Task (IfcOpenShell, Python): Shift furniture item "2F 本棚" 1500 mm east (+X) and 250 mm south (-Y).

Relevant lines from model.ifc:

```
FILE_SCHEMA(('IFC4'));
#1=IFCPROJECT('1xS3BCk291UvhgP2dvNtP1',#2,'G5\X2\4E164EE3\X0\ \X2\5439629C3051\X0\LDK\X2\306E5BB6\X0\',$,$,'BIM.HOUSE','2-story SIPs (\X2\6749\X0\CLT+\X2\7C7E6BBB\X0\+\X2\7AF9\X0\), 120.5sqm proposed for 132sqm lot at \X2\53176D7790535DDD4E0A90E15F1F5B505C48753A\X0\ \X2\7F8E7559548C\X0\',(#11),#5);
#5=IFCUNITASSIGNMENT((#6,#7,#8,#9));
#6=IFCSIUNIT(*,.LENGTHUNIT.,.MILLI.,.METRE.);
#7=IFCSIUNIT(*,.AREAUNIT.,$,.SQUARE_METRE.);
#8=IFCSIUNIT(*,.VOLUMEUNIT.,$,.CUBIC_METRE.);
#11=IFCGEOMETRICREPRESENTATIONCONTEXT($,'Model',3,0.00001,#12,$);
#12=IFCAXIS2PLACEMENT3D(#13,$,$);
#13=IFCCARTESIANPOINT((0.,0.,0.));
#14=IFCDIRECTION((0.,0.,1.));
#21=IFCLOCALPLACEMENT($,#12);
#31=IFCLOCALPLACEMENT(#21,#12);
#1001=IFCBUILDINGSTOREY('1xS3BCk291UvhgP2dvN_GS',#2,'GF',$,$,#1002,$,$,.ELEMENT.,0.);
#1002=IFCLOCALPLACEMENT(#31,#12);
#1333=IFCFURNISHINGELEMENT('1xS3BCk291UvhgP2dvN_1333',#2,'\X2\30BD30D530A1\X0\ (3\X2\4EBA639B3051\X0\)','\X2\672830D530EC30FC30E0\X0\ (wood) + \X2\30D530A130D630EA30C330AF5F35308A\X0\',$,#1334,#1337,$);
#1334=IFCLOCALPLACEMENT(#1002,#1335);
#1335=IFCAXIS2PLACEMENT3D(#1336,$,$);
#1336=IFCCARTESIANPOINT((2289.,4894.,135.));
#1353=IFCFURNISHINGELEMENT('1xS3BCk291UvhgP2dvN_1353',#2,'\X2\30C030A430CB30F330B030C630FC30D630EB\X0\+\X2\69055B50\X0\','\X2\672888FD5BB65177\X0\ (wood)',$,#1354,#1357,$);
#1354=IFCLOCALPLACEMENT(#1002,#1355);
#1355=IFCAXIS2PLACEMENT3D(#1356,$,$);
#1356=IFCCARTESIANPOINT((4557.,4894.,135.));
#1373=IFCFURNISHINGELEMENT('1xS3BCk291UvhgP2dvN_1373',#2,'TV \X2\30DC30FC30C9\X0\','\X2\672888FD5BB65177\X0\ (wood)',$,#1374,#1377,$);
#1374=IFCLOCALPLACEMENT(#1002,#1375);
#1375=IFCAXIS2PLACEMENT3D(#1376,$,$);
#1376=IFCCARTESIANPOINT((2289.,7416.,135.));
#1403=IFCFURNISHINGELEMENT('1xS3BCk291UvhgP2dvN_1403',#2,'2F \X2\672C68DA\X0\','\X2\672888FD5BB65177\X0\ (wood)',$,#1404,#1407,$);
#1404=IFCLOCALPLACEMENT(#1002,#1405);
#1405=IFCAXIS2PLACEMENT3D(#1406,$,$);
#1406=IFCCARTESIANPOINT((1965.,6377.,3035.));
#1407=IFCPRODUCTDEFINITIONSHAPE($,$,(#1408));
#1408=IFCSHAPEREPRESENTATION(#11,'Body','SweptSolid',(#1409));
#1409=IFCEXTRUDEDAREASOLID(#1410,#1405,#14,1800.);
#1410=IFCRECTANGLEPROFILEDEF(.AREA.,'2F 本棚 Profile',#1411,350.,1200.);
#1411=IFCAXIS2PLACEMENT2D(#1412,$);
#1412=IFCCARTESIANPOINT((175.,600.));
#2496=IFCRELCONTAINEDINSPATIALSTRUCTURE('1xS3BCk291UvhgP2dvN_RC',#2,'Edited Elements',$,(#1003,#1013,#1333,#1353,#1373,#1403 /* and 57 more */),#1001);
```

```python
import ifcopenshell
import ifcopenshell.api.geometry
import ifcopenshell.util.placement

model = ifcopenshell.open("model.ifc")

item = model.by_guid("1xS3BCk291UvhgP2dvN_1403")
matrix = ifcopenshell.util.placement.get_local_placement(item.ObjectPlacement)
matrix[0, 3] += 1500.0
matrix[1, 3] -= 250.0
ifcopenshell.api.geometry.edit_object_placement(model, product=item, matrix=matrix, is_si=False)

print(ifcopenshell.util.placement.get_local_placement(item.ObjectPlacement).round(3) + 0.0)

model.write("model_updated.ifc")
```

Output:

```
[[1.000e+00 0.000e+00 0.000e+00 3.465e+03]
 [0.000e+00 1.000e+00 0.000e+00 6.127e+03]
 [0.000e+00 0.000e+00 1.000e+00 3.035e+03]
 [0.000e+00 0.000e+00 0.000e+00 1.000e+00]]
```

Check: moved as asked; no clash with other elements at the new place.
